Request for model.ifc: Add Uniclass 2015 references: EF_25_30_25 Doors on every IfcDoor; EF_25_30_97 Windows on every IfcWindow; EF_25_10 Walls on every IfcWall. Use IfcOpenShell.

First a look at what the model holds.

```python
import ifcopenshell

model = ifcopenshell.open("model.ifc")
print(model.schema)
print("classifications:", [c.Name for c in model.by_type("IfcClassification")])
for ifc_class in ("IfcDoor", "IfcRoof", "IfcStair", "IfcWall", "IfcWindow"):
    print(ifc_class, len(model.by_type(ifc_class)))
```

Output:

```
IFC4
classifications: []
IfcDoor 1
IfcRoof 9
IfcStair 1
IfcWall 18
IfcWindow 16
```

```python
import ifcopenshell
import ifcopenshell.api.classification

model = ifcopenshell.open("model.ifc")

system = ifcopenshell.api.classification.add_classification(model, classification="Uniclass 2015")

codes = {
    "IfcDoor": ("EF_25_30_25", "Doors"),
    "IfcWindow": ("EF_25_30_97", "Windows"),
    "IfcWall": ("EF_25_10", "Walls"),
}
for ifc_class, (code, name) in codes.items():
    products = model.by_type(ifc_class)
    ifcopenshell.api.classification.add_reference(
        model, products=products, classification=system, identification=code, name=name
    )
    print(code, len(products))

model.write("model_v2.ifc")
```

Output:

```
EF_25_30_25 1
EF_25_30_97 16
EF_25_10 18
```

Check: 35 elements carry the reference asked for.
